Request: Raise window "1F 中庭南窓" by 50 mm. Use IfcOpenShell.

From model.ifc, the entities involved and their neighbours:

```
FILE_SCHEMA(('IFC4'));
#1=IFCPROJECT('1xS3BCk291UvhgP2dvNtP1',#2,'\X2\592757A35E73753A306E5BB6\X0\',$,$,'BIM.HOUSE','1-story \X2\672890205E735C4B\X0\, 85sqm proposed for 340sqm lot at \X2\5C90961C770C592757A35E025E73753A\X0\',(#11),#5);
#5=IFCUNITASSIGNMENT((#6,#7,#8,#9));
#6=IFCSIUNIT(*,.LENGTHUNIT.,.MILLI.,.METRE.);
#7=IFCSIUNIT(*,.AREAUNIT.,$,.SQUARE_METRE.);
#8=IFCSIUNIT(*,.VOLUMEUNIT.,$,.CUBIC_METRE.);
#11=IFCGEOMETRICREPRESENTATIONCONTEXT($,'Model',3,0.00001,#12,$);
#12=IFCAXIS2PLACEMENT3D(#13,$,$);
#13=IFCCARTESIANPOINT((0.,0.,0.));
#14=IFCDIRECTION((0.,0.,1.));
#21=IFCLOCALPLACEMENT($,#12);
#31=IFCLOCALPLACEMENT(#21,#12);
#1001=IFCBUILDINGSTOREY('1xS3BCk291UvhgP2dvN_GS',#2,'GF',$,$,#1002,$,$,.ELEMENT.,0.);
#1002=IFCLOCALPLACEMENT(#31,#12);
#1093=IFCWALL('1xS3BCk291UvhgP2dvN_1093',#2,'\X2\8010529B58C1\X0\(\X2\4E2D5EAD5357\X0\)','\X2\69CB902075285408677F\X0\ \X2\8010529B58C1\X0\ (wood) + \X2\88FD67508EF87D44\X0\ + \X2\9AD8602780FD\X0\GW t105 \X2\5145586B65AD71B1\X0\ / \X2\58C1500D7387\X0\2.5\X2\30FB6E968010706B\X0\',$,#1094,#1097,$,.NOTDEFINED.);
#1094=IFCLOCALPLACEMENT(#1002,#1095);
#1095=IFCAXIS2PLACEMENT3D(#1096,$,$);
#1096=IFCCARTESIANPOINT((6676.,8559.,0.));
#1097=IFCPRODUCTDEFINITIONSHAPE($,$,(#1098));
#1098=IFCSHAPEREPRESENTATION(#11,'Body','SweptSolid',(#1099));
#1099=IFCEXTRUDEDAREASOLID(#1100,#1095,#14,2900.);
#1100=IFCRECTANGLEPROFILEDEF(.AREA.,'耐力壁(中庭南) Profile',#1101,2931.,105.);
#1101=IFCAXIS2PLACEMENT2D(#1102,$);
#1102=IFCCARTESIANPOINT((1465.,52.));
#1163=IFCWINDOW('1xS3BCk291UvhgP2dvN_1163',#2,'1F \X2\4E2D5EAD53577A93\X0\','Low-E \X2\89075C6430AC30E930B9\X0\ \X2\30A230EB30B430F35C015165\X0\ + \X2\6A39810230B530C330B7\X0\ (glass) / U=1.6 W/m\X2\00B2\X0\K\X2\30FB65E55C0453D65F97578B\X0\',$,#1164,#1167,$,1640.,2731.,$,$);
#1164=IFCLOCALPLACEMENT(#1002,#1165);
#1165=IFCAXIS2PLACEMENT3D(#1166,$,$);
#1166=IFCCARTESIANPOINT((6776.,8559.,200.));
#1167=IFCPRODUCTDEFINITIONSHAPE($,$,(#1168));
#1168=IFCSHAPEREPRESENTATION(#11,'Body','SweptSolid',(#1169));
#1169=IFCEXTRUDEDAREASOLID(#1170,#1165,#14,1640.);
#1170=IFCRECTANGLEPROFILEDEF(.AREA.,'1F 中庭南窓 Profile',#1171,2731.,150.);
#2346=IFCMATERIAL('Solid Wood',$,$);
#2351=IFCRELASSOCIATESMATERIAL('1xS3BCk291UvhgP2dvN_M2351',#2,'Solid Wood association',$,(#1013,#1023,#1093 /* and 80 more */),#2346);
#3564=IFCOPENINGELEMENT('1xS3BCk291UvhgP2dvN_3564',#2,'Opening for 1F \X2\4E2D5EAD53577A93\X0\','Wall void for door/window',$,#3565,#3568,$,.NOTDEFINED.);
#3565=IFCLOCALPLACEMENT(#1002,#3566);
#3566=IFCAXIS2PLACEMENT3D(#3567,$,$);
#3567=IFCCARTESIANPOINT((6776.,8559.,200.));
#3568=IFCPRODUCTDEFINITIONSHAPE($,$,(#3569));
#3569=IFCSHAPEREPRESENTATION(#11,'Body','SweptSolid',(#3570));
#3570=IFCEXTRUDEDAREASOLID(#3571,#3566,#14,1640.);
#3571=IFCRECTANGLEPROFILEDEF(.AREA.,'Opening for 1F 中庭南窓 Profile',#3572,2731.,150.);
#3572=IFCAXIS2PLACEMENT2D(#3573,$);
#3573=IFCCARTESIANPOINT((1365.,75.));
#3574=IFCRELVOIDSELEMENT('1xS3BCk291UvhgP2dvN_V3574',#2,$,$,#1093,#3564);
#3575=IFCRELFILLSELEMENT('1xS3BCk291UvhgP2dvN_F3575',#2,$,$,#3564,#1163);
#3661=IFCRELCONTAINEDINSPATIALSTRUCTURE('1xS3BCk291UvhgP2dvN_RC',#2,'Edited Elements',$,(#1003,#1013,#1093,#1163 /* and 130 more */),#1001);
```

```python
import numpy as np
import ifcopenshell
import ifcopenshell.api.geometry
import ifcopenshell.util.placement
import ifcopenshell.util.unit

model = ifcopenshell.open("model.ifc")
unit_scale = ifcopenshell.util.unit.calculate_unit_scale(model)

window = model.by_id(1163)
opening = window.FillsVoids[0].RelatingOpeningElement
dz = 0.05 / unit_scale

shift = np.array([0.0, 0.0, dz])
# The window is not placed relative to its opening, so move both.
for product in (opening, window):
    matrix = ifcopenshell.util.placement.get_local_placement(product.ObjectPlacement)
    matrix[:3, 3] += shift
    ifcopenshell.api.geometry.edit_object_placement(model, product=product, matrix=matrix, is_si=False)

print(f"moved by {dz * unit_scale:+.3f} m")

model.write("model_edited.ifc")
```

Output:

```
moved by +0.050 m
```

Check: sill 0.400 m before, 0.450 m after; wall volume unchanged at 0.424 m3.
